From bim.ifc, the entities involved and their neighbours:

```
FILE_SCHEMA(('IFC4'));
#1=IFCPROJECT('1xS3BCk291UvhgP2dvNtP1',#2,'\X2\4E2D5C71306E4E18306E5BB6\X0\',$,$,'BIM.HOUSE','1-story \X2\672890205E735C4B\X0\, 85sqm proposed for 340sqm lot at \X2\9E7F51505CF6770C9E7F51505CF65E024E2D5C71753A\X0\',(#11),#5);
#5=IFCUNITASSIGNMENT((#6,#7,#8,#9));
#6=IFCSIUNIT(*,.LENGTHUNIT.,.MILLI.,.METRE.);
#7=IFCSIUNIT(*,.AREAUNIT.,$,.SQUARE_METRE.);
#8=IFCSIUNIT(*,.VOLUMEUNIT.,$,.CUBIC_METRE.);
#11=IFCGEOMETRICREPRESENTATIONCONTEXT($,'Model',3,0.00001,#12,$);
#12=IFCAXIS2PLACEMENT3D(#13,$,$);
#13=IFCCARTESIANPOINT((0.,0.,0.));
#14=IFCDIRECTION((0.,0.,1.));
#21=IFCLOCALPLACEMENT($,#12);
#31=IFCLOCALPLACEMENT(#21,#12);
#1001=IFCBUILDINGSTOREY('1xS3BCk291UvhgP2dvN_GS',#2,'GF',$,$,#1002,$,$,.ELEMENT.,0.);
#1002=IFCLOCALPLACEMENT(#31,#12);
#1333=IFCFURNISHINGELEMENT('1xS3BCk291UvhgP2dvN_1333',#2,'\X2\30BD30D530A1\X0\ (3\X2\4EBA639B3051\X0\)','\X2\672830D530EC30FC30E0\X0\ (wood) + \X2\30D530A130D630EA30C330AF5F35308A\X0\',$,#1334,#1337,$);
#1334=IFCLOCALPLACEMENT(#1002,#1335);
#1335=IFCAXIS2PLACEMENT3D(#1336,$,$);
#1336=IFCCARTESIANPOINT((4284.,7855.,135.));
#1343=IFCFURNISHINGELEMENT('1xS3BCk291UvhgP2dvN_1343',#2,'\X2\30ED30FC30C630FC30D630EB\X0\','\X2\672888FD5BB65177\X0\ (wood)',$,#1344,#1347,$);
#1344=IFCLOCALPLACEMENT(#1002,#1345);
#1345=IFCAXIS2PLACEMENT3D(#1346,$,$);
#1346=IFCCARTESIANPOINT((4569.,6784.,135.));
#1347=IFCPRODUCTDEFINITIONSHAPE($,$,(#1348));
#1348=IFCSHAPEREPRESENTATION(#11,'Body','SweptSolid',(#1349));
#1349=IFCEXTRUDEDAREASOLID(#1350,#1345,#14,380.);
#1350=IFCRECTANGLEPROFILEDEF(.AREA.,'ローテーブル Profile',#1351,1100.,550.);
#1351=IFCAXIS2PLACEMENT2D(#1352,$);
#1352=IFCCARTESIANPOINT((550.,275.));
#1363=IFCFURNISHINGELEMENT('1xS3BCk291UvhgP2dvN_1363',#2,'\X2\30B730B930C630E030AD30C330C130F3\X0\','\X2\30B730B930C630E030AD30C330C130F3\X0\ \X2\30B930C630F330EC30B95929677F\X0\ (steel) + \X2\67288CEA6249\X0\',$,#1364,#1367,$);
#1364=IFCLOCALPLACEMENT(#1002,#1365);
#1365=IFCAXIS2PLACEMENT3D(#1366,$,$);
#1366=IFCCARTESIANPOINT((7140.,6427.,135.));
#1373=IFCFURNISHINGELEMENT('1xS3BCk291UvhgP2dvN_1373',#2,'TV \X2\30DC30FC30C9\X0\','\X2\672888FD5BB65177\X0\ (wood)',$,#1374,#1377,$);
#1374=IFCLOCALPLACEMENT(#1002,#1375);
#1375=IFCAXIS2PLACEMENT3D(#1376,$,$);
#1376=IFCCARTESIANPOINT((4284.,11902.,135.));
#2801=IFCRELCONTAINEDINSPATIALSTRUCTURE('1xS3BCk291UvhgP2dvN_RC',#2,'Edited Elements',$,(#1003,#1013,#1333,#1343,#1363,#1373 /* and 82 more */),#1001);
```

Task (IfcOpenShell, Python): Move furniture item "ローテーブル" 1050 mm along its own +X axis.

```python
import ifcopenshell
import ifcopenshell.api.geometry
import ifcopenshell.util.placement
import ifcopenshell.util.unit

model = ifcopenshell.open("bim.ifc")
unit_scale = ifcopenshell.util.unit.calculate_unit_scale(model)

item = model.by_id(1343)
matrix = ifcopenshell.util.placement.get_local_placement(item.ObjectPlacement)
matrix[:3, 3] += matrix[:3, 0] * 1.05 / unit_scale
ifcopenshell.api.geometry.edit_object_placement(model, product=item, matrix=matrix, is_si=False)

print(ifcopenshell.util.placement.get_local_placement(item.ObjectPlacement).round(3) + 0.0)

model.write("bim_updated.ifc")
```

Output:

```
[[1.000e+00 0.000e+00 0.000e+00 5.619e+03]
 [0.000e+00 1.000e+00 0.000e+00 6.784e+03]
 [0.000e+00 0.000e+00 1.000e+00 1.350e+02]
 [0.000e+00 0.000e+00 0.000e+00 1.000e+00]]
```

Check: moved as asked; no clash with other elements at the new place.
